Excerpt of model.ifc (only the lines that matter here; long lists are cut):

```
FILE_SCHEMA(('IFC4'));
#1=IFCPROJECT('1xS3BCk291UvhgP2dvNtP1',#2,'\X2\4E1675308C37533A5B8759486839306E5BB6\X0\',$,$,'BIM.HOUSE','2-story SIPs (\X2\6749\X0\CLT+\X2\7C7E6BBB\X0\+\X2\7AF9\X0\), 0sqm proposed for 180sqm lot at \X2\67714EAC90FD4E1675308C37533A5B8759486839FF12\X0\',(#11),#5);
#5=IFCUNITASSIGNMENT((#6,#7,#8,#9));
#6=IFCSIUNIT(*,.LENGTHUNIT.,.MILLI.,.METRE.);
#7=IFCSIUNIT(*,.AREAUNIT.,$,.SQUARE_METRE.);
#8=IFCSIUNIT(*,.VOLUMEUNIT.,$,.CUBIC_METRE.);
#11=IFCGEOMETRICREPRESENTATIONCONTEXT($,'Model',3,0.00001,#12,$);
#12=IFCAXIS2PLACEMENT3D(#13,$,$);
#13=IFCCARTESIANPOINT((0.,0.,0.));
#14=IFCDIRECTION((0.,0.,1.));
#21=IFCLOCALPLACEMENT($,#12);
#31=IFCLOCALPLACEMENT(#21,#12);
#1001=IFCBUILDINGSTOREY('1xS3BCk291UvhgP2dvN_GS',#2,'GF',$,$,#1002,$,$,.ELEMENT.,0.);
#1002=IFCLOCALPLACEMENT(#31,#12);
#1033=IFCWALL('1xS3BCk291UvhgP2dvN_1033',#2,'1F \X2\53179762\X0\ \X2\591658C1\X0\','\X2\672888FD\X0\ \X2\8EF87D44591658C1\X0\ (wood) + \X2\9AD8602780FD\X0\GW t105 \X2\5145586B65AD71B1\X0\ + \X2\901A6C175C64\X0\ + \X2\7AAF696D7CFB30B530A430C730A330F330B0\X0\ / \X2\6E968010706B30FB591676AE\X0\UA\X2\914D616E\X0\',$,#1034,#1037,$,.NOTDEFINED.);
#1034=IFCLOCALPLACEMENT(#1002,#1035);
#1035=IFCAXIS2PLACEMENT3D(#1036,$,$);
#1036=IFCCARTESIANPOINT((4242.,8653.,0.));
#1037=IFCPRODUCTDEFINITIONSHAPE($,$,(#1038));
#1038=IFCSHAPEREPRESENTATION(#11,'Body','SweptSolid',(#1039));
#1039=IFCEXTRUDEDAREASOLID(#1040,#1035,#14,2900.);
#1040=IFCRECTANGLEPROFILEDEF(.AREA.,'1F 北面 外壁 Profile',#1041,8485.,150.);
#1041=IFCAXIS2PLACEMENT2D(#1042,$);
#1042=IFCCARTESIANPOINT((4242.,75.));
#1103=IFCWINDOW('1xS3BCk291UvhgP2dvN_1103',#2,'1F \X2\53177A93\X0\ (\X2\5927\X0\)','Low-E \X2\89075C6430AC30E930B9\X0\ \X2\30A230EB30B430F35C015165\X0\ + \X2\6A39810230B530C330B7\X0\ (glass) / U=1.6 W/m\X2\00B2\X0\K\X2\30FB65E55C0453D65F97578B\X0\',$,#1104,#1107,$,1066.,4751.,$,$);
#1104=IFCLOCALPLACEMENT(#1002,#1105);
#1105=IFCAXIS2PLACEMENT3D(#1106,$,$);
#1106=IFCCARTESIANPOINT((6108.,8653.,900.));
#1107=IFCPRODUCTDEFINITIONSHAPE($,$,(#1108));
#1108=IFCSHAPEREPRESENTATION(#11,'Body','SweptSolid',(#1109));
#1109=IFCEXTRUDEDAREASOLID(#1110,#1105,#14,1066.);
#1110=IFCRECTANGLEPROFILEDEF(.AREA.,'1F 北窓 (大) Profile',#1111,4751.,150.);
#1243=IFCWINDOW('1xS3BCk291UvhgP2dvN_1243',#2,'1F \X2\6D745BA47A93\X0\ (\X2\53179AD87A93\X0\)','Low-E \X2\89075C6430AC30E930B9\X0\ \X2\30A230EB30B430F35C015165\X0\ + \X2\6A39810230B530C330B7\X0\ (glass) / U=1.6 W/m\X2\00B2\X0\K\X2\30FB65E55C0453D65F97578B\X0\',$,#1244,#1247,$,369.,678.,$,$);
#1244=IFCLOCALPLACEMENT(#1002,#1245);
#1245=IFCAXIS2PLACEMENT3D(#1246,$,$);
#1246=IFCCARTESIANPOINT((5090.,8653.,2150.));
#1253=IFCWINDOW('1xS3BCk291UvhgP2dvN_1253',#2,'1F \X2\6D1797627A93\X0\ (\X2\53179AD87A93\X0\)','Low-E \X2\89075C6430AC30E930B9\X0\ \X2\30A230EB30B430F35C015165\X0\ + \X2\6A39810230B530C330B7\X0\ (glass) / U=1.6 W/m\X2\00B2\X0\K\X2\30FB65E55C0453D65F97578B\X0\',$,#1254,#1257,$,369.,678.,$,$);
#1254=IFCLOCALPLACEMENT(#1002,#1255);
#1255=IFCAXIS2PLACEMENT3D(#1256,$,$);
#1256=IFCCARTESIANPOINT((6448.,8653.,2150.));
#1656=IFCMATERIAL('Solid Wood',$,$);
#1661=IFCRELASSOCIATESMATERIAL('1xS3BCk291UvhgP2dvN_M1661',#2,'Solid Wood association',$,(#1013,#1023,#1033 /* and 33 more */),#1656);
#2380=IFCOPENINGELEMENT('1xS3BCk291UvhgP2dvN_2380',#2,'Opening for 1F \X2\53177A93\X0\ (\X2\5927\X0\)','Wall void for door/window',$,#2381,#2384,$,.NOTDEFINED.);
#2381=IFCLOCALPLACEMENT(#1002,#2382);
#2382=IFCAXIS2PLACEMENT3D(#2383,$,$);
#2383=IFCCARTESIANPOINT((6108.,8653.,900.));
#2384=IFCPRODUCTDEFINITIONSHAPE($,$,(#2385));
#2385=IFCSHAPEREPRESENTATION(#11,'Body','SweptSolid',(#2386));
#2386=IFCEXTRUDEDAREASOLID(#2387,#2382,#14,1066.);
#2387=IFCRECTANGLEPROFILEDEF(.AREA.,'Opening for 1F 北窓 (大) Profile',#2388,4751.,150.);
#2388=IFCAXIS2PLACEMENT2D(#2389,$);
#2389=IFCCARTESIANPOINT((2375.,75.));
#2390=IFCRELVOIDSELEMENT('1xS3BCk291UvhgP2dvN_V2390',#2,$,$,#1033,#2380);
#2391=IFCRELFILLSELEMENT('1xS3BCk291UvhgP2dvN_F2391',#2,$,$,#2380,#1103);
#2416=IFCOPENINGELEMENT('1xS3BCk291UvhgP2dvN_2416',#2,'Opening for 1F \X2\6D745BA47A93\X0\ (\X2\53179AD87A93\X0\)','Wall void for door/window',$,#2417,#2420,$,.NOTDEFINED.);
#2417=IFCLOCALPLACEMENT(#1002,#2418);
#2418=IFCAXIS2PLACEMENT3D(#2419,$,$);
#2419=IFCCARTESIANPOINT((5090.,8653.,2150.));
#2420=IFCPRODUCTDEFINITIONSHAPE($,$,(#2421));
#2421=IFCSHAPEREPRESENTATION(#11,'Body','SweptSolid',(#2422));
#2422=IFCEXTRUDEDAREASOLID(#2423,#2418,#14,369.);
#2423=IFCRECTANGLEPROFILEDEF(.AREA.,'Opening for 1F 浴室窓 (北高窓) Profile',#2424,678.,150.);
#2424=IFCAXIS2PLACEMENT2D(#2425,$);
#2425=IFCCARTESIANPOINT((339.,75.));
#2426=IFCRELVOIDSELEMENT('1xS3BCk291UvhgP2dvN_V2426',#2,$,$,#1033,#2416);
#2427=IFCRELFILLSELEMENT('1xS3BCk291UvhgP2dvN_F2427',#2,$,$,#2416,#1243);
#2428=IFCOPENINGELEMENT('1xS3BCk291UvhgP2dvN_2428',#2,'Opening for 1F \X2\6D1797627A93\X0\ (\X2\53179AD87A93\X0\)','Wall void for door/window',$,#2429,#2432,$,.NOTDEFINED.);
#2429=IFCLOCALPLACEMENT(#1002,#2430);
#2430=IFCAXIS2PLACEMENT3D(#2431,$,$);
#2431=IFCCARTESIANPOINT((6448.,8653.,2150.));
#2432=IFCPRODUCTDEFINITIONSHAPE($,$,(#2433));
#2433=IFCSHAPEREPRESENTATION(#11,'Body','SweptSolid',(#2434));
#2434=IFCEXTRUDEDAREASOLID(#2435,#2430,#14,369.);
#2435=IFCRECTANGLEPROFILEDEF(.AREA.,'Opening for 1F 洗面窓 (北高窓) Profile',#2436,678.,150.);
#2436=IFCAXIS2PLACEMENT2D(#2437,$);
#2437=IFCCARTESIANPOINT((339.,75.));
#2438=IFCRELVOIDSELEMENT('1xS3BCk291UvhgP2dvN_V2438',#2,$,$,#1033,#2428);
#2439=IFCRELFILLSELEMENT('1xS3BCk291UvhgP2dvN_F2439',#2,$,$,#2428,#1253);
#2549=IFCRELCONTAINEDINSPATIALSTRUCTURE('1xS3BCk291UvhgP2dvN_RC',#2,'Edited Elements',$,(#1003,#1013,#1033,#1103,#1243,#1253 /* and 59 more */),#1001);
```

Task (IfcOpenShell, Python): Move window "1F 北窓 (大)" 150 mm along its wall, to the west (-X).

```python
import ifcopenshell
import ifcopenshell.api.geometry
import ifcopenshell.util.placement

model = ifcopenshell.open("model.ifc")

window = model.by_guid("1xS3BCk291UvhgP2dvN_1103")
opening = window.FillsVoids[0].RelatingOpeningElement
wall = opening.VoidsElements[0].RelatingBuildingElement

wall_matrix = ifcopenshell.util.placement.get_local_placement(wall.ObjectPlacement)
shift = wall_matrix[:3, 0] * -150.0
before = ifcopenshell.util.placement.get_local_placement(window.ObjectPlacement)[:3, 3].copy()

# The window is not placed relative to its opening, so move both.
for product in (opening, window):
    matrix = ifcopenshell.util.placement.get_local_placement(product.ObjectPlacement)
    matrix[:3, 3] += shift
    ifcopenshell.api.geometry.edit_object_placement(model, product=product, matrix=matrix, is_si=False)

after = ifcopenshell.util.placement.get_local_placement(window.ObjectPlacement)[:3, 3]
print("window moved by", (after - before).round(3) + 0.0)

model.write("model_rev.ifc")
```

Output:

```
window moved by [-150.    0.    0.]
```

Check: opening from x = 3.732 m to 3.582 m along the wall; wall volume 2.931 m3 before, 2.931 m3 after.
